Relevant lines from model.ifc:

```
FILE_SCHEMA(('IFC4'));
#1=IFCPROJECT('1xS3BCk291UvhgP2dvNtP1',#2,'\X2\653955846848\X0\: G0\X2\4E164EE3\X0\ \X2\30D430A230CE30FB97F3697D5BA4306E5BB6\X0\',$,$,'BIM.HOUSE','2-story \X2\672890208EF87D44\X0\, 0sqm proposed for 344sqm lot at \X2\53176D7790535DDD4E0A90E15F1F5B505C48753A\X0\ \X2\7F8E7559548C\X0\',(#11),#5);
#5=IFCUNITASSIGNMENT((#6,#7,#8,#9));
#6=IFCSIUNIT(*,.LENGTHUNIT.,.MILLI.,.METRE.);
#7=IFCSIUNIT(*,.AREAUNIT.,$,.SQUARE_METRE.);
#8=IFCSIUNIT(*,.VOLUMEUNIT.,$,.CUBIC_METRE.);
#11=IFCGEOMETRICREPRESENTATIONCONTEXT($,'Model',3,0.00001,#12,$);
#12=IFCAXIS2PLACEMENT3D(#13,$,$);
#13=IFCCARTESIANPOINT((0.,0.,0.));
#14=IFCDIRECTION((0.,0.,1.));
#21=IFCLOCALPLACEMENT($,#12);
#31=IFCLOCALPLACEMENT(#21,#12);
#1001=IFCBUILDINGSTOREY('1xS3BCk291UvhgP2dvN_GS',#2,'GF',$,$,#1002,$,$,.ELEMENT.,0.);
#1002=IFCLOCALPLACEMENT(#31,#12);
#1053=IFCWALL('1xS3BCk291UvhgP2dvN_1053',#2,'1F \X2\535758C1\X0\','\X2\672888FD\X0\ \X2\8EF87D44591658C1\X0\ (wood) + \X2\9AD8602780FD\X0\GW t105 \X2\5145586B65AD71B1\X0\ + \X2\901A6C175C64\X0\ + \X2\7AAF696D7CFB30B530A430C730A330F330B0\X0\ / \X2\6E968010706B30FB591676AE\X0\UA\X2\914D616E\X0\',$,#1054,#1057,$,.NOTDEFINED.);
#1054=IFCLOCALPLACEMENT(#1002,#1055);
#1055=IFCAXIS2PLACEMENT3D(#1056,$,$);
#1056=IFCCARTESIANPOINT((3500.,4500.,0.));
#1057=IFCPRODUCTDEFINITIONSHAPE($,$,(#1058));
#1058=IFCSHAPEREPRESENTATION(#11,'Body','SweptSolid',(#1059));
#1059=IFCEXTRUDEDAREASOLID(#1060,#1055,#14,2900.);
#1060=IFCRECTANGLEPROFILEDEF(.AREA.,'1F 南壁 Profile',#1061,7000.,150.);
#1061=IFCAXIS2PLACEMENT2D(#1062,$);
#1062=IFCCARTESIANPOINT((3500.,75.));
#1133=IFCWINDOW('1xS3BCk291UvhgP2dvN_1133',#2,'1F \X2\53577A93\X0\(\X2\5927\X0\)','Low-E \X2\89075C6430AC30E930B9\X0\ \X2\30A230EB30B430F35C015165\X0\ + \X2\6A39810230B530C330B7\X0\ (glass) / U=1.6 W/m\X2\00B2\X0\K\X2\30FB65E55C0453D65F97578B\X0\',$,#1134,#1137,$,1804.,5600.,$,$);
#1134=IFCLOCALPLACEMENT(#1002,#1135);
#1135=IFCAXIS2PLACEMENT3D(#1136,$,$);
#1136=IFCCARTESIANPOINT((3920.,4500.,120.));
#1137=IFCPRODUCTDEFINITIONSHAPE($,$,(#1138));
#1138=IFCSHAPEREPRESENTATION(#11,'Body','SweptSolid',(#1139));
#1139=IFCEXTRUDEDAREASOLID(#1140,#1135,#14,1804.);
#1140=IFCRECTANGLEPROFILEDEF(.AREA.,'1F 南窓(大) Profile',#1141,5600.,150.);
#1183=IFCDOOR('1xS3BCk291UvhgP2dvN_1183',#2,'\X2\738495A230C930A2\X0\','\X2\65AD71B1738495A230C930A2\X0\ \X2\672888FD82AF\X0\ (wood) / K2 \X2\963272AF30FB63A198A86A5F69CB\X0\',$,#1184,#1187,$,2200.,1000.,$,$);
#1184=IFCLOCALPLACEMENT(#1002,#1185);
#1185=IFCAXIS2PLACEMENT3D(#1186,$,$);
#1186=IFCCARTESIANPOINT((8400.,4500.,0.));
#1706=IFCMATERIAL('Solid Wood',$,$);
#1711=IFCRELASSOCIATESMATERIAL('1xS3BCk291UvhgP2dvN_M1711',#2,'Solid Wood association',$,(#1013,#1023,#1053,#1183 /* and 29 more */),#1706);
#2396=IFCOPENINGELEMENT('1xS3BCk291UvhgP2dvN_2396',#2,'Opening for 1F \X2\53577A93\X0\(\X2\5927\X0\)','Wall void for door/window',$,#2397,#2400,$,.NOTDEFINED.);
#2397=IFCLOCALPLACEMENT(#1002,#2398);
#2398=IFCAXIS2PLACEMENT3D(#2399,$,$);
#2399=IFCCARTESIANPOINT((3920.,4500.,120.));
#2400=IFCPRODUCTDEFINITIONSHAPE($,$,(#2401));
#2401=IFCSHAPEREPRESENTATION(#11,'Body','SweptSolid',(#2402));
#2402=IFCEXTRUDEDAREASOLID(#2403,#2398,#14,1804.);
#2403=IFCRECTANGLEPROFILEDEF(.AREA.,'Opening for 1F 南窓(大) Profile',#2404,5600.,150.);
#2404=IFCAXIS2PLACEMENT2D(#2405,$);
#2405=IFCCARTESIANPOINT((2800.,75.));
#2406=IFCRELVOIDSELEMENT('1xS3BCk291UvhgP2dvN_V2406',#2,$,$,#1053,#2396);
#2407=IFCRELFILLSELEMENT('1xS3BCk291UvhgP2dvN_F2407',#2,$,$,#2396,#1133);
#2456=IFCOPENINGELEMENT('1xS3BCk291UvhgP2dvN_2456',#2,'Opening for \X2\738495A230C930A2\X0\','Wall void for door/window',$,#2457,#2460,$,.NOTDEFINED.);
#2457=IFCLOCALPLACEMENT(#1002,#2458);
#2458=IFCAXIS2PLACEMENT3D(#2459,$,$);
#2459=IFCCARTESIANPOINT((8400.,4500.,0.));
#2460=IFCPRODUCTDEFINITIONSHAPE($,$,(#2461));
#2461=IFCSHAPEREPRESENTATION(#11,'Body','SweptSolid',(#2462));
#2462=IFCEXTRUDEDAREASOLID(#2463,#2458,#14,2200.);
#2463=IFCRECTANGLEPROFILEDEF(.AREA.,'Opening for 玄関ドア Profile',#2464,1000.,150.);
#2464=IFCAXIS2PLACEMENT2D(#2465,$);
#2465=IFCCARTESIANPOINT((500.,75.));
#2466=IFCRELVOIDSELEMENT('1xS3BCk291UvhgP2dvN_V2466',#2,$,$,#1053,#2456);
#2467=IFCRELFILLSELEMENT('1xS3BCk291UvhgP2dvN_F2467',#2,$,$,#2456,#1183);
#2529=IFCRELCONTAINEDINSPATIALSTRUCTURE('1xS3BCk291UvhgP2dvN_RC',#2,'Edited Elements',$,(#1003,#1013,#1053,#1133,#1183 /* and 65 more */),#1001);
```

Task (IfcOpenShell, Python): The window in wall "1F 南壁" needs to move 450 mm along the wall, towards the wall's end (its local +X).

```python
import ifcopenshell
import ifcopenshell.api.geometry
import ifcopenshell.util.placement
import ifcopenshell.util.unit

model = ifcopenshell.open("model.ifc")
unit_scale = ifcopenshell.util.unit.calculate_unit_scale(model)

window = model.by_guid("1xS3BCk291UvhgP2dvN_1133")
opening = window.FillsVoids[0].RelatingOpeningElement
wall = opening.VoidsElements[0].RelatingBuildingElement

wall_matrix = ifcopenshell.util.placement.get_local_placement(wall.ObjectPlacement)
shift = wall_matrix[:3, 0] * 0.45 / unit_scale
before = ifcopenshell.util.placement.get_local_placement(window.ObjectPlacement)[:3, 3].copy()

# The window is not placed relative to its opening, so move both.
for product in (opening, window):
    matrix = ifcopenshell.util.placement.get_local_placement(product.ObjectPlacement)
    matrix[:3, 3] += shift
    ifcopenshell.api.geometry.edit_object_placement(model, product=product, matrix=matrix, is_si=False)

after = ifcopenshell.util.placement.get_local_placement(window.ObjectPlacement)[:3, 3]
print("window moved by", (after - before).round(3) + 0.0)

model.write("model_rev.ifc")
```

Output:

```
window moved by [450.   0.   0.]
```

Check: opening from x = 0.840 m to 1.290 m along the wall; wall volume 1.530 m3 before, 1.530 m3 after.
